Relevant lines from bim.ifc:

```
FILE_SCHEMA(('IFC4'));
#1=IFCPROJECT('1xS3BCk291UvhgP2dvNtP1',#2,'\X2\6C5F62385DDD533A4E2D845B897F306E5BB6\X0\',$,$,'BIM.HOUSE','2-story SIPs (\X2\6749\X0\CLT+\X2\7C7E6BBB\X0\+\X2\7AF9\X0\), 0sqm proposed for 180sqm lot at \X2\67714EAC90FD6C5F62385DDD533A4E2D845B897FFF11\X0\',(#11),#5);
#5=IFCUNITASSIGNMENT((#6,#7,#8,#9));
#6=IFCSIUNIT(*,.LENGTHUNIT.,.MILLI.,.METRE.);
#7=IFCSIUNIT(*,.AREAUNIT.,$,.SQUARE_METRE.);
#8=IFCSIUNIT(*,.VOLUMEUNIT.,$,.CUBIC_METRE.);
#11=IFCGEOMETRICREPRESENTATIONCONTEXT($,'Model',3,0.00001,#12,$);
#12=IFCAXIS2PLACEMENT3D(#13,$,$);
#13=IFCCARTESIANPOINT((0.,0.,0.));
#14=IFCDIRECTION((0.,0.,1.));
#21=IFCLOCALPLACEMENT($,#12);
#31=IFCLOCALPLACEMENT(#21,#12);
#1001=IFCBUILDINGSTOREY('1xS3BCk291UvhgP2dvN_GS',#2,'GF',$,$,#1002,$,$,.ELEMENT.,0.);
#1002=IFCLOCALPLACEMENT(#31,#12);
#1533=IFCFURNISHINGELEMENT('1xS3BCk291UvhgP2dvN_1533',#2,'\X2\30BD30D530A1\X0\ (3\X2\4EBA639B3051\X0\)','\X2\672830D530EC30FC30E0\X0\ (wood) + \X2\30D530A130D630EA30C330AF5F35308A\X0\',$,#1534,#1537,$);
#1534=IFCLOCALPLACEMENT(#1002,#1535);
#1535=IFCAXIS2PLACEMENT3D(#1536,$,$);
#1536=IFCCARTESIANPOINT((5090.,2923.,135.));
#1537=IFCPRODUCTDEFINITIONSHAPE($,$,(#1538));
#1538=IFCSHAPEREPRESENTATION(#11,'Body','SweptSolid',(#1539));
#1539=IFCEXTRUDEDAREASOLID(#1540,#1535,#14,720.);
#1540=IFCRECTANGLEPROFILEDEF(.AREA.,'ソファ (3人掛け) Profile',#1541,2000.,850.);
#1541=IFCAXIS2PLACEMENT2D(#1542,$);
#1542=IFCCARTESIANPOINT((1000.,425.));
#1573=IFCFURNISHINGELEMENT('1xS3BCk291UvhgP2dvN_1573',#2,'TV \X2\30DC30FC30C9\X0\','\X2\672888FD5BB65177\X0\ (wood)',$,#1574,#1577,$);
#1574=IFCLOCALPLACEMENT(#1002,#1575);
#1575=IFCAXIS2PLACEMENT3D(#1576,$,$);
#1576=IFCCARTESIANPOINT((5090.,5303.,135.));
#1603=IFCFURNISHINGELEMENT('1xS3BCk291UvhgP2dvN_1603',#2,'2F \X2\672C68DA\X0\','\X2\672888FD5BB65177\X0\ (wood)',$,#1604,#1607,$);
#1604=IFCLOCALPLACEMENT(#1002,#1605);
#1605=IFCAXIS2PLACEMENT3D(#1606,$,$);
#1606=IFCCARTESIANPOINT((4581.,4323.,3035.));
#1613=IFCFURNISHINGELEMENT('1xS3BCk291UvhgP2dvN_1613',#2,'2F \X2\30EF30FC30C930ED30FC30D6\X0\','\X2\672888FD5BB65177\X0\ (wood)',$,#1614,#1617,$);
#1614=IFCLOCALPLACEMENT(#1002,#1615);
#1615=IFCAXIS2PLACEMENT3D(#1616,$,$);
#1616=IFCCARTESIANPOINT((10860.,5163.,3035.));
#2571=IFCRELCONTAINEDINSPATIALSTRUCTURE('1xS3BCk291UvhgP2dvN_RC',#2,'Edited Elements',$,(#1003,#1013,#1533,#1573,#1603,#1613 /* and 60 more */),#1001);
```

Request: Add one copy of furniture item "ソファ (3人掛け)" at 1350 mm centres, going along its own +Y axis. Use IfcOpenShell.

```python
import ifcopenshell
import ifcopenshell.api.geometry
import ifcopenshell.api.root
import ifcopenshell.util.element
import ifcopenshell.util.placement
import ifcopenshell.util.unit

model = ifcopenshell.open("bim.ifc")
unit_scale = ifcopenshell.util.unit.calculate_unit_scale(model)


def reuse_history(source, copy):
    """copy_class also copies each property set's owner history, people and application; keep the originals."""
    for rel in copy.IsDefinedBy:
        if rel.is_a("IfcRelDefinesByProperties") and (history := rel.RelatingPropertyDefinition.OwnerHistory):
            rel.RelatingPropertyDefinition.OwnerHistory = source.OwnerHistory
            ifcopenshell.util.element.remove_deep2(model, history)


source = model.by_guid("1xS3BCk291UvhgP2dvN_1533")
base = ifcopenshell.util.placement.get_local_placement(source.ObjectPlacement)
step = base[:3, 1] * 1.35 / unit_scale

for i in range(1, 2):
    copy = ifcopenshell.api.root.copy_class(model, product=source)
    copy.Representation = ifcopenshell.util.element.copy_deep(
        model, source.Representation, exclude=["IfcGeometricRepresentationContext", "IfcRepresentationMap"]
    )
    reuse_history(source, copy)
    matrix = base.copy()
    matrix[:3, 3] += i * step
    print("added at", matrix[:3, 3].round(3) + 0.0)
    ifcopenshell.api.geometry.edit_object_placement(model, product=copy, matrix=matrix, is_si=False)

model.write("bim_rev.ifc")
```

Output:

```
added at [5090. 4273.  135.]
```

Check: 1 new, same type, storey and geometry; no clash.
